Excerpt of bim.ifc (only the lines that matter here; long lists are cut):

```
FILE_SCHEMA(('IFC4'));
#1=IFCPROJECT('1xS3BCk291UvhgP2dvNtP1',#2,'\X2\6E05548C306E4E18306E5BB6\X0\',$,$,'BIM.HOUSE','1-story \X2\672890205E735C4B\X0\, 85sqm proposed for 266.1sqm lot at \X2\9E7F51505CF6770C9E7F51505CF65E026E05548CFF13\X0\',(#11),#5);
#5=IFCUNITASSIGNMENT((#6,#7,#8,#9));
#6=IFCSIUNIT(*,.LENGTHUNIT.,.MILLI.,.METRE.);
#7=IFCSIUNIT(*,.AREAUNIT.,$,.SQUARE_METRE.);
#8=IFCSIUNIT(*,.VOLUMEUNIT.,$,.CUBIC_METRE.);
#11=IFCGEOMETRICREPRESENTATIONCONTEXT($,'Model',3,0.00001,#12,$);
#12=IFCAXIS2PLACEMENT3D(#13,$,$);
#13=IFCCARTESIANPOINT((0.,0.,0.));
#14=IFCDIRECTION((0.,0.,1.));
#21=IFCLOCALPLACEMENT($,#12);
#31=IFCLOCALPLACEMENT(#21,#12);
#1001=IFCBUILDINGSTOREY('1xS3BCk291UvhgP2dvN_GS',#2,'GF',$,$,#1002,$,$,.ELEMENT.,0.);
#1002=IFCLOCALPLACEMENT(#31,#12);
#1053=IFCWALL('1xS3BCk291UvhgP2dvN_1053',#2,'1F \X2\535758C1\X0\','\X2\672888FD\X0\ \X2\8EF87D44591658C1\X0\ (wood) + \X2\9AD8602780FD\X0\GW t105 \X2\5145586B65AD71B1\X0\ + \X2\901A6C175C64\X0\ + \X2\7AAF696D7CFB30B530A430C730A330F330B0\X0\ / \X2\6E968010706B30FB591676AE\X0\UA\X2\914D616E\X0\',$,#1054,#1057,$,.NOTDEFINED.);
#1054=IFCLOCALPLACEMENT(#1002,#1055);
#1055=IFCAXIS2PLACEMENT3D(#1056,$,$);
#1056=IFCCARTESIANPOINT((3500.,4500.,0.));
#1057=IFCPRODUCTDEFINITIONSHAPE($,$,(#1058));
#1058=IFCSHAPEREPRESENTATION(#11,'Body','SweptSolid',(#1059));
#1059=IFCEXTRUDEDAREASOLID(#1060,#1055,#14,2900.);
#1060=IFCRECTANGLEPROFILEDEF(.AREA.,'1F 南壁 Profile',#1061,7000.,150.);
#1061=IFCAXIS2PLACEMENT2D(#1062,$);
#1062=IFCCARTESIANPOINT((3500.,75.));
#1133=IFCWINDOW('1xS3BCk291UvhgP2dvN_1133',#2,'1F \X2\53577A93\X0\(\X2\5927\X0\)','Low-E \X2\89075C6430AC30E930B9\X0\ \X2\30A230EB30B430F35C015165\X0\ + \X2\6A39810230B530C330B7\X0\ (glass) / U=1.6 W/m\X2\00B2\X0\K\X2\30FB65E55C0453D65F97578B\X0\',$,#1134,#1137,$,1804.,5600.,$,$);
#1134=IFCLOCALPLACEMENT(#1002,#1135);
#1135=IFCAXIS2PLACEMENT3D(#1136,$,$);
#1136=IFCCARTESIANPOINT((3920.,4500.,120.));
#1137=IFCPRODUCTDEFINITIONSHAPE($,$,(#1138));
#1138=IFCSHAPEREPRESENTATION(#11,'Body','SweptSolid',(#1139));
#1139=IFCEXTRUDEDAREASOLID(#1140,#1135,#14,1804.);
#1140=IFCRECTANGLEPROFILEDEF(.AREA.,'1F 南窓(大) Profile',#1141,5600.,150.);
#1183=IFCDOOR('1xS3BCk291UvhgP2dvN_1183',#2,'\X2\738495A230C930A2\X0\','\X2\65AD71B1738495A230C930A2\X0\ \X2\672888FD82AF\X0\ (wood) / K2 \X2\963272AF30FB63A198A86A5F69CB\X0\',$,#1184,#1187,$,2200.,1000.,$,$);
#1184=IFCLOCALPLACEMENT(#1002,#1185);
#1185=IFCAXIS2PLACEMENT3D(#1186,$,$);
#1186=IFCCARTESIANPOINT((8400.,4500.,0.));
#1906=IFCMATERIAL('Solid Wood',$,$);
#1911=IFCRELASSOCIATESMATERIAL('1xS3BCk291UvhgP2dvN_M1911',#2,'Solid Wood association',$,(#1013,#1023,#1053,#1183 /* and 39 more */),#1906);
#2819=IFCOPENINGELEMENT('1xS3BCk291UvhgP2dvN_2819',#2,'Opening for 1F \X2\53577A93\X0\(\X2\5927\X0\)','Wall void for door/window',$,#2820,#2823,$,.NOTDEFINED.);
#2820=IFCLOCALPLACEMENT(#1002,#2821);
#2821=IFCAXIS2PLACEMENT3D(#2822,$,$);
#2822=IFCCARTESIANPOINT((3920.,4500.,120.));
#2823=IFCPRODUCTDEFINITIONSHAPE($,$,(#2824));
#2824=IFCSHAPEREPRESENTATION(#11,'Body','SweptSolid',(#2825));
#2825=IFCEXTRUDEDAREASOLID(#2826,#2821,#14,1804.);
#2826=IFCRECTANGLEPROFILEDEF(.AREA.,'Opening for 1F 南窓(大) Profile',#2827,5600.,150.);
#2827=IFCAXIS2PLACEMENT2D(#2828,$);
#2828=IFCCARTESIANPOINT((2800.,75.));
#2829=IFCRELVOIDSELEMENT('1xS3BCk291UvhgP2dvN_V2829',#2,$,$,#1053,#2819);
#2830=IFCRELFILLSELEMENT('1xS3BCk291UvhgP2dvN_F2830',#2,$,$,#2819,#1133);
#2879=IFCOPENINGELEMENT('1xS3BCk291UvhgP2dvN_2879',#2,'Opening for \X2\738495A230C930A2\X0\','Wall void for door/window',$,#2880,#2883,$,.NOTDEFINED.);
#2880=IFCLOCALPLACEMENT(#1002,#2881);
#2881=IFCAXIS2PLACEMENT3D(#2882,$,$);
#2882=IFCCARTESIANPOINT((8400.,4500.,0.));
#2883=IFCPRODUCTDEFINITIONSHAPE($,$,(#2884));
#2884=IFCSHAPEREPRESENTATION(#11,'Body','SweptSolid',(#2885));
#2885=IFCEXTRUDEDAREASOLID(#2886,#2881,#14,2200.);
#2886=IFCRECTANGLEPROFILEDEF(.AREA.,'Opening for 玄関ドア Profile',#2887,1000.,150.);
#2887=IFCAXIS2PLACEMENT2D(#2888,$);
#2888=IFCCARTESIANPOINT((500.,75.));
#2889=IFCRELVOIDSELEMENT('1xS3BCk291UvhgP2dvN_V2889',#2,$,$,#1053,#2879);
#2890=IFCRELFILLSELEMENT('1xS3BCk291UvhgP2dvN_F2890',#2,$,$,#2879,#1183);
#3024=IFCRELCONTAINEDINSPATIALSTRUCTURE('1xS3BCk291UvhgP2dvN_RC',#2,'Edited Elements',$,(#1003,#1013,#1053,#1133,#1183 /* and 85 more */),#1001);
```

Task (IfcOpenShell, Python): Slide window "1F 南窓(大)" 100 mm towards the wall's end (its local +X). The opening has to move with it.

```python
import ifcopenshell
import ifcopenshell.api.geometry
import ifcopenshell.util.placement

model = ifcopenshell.open("bim.ifc")

window = model.by_guid("1xS3BCk291UvhgP2dvN_1133")
opening = window.FillsVoids[0].RelatingOpeningElement
wall = opening.VoidsElements[0].RelatingBuildingElement

wall_matrix = ifcopenshell.util.placement.get_local_placement(wall.ObjectPlacement)
shift = wall_matrix[:3, 0] * 100.0
before = ifcopenshell.util.placement.get_local_placement(window.ObjectPlacement)[:3, 3].copy()

# The window is not placed relative to its opening, so move both.
for product in (opening, window):
    matrix = ifcopenshell.util.placement.get_local_placement(product.ObjectPlacement)
    matrix[:3, 3] += shift
    ifcopenshell.api.geometry.edit_object_placement(model, product=product, matrix=matrix, is_si=False)

after = ifcopenshell.util.placement.get_local_placement(window.ObjectPlacement)[:3, 3]
print("window moved by", (after - before).round(3) + 0.0)

model.write("bim_v2.ifc")
```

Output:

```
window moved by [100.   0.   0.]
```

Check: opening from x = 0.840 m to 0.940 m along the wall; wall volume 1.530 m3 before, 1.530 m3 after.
